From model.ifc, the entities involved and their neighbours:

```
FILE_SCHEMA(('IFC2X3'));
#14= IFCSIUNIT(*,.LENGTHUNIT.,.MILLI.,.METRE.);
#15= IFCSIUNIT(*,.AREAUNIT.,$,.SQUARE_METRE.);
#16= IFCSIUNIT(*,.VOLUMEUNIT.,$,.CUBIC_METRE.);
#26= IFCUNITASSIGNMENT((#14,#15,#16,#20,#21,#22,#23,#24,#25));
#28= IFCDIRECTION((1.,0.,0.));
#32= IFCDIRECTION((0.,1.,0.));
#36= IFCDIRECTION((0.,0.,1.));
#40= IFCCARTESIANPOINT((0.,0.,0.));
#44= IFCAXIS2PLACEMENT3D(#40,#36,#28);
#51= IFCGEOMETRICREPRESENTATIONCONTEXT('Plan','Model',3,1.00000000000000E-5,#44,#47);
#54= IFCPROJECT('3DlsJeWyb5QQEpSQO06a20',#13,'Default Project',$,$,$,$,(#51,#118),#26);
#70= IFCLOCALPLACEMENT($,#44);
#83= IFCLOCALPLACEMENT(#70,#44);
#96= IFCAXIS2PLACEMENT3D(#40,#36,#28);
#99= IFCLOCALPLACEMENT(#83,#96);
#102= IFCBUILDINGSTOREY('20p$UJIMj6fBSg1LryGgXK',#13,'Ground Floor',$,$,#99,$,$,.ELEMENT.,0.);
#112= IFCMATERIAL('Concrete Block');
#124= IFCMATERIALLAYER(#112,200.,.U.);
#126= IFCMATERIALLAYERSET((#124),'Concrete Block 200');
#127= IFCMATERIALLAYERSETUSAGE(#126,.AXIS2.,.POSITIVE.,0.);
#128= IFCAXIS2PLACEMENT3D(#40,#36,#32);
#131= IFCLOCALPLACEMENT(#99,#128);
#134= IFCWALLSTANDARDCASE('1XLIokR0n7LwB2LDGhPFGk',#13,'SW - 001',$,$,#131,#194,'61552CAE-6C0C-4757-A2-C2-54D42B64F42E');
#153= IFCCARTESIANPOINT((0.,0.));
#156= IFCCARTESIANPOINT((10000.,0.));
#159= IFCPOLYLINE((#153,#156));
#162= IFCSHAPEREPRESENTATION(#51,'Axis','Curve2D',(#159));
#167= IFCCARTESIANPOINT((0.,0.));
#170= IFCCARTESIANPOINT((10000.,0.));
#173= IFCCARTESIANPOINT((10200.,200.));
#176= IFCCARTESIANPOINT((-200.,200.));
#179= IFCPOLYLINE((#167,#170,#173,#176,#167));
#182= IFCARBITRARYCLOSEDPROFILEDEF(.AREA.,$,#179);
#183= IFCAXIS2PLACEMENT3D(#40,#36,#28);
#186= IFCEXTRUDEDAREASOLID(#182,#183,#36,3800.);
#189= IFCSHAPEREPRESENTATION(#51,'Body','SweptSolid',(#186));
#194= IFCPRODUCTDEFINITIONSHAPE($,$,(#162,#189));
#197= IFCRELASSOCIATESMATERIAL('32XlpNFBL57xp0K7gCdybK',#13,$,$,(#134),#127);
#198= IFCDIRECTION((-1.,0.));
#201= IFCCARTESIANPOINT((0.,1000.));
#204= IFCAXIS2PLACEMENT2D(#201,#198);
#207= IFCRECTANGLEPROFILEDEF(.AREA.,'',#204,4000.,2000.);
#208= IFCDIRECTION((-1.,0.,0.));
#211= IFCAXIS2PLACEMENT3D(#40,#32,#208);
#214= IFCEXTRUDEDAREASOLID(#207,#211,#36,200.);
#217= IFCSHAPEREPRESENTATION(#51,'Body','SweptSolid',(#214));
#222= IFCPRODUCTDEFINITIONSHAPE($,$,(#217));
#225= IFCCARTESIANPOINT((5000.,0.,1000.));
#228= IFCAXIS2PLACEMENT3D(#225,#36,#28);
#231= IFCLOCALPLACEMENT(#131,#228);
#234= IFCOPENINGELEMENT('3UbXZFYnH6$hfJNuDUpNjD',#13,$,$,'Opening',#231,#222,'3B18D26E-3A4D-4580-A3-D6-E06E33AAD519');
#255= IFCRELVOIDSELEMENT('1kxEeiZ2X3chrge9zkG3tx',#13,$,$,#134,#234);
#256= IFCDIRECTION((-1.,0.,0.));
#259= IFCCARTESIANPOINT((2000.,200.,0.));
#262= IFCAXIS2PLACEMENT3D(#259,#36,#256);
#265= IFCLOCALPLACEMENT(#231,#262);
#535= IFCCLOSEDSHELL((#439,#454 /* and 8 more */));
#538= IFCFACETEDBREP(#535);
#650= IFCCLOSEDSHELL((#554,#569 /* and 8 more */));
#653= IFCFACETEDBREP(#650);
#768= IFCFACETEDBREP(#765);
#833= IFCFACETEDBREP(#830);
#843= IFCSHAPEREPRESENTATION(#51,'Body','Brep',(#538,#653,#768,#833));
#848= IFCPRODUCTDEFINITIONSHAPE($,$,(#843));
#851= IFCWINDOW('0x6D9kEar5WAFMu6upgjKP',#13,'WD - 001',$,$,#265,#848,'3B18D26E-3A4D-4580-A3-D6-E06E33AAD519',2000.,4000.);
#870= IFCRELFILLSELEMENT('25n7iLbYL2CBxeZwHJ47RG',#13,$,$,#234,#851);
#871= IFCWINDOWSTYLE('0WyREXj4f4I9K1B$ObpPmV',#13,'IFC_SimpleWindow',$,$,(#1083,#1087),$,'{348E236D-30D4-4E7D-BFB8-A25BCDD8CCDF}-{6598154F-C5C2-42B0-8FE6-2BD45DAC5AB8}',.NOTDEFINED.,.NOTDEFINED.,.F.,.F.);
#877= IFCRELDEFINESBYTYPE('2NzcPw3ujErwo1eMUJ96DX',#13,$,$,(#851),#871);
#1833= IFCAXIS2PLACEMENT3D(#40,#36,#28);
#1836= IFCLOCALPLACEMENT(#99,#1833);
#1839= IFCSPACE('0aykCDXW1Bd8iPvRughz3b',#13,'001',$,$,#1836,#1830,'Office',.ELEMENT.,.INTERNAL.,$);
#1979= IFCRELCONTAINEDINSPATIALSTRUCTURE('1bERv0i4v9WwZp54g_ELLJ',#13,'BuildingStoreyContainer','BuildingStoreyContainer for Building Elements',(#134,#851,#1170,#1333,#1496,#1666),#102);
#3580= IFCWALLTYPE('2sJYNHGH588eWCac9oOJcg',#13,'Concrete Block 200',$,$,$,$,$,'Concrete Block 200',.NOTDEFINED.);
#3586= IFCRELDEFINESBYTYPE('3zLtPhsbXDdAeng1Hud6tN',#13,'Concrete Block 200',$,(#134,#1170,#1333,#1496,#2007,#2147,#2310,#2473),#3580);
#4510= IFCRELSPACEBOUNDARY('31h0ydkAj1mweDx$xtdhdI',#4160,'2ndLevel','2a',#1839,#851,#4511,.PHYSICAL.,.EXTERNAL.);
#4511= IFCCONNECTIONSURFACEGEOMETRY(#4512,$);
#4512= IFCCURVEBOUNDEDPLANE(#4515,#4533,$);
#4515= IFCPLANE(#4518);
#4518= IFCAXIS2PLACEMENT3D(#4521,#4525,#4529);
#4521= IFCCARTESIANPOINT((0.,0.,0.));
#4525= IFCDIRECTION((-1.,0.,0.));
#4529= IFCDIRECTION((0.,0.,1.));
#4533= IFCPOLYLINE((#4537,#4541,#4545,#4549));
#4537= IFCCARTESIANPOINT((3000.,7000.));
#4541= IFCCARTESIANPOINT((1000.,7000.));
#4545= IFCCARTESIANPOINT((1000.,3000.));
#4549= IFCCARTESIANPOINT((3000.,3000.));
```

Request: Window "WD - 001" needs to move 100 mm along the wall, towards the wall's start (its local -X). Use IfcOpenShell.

```python
import numpy as np
import ifcopenshell
import ifcopenshell.api.geometry
import ifcopenshell.util.placement
import ifcopenshell.util.unit

model = ifcopenshell.open("model.ifc")
unit_scale = ifcopenshell.util.unit.calculate_unit_scale(model)

window = model.by_guid("0x6D9kEar5WAFMu6upgjKP")
opening = window.FillsVoids[0].RelatingOpeningElement
wall = opening.VoidsElements[0].RelatingBuildingElement

wall_matrix = ifcopenshell.util.placement.get_local_placement(wall.ObjectPlacement)
shift = wall_matrix[:3, 0] * -0.1 / unit_scale
before = ifcopenshell.util.placement.get_local_placement(window.ObjectPlacement)[:3, 3].copy()

# The window is placed relative to its opening, so it follows when the opening moves.
matrix = ifcopenshell.util.placement.get_local_placement(opening.ObjectPlacement)
matrix[:3, 3] += shift
ifcopenshell.api.geometry.edit_object_placement(
    model, product=opening, matrix=matrix, is_si=False, should_transform_children=True
)

# Space boundary surfaces are stored in each space's coordinates; move them too.
for rel in window.ProvidesBoundaries:
    if not rel.ConnectionGeometry:
        continue
    surface = rel.ConnectionGeometry.SurfaceOnRelatingElement.BasisSurface
    space_matrix = ifcopenshell.util.placement.get_local_placement(rel.RelatingSpace.ObjectPlacement)
    point = np.array(surface.Position.Location.Coordinates) + space_matrix[:3, :3].T @ shift
    surface.Position = model.createIfcAxis2Placement3D(
        model.createIfcCartesianPoint(point.tolist()), surface.Position.Axis, surface.Position.RefDirection
    )

after = ifcopenshell.util.placement.get_local_placement(window.ObjectPlacement)[:3, 3]
print("window moved by", (after - before).round(3) + 0.0)

model.write("model_rev.ifc")
```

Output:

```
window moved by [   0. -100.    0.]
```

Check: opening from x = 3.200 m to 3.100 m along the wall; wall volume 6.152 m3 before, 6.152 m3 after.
